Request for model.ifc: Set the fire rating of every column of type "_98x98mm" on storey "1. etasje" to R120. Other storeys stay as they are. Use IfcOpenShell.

First a look at what the model holds.

```python
import ifcopenshell
import ifcopenshell.util.element

model = ifcopenshell.open("model.ifc")
print(model.schema)
storey = next(s for s in model.by_type("IfcBuildingStorey") if s.Name == "1. etasje")
columns = [e for e in ifcopenshell.util.element.get_decomposition(storey) if e.is_a("IfcColumn")]
seen = {}
for e in columns:
    element_type = ifcopenshell.util.element.get_type(e)
    key = (element_type.Name if element_type != e and element_type else None, ifcopenshell.util.element.get_pset(e, "Pset_ColumnCommon", "FireRating"))
    seen[key] = seen.get(key, 0) + 1
for (name, value), count in sorted(seen.items(), key=str):
    print(count, "x", name, "|", value)
```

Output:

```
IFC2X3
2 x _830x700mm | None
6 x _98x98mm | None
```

```python
import ifcopenshell
import ifcopenshell.api.pset
import ifcopenshell.util.element

model = ifcopenshell.open("model.ifc")

storey = next(s for s in model.by_type("IfcBuildingStorey") if s.Name == "1. etasje")
columns = [e for e in ifcopenshell.util.element.get_decomposition(storey) if e.is_a("IfcColumn")]

count = 0
for e in columns:
    element_type = ifcopenshell.util.element.get_type(e)
    if element_type in (None, e) or element_type.Name != "_98x98mm":
        continue
    # add_pset returns the element's existing set when there is one.
    pset = ifcopenshell.api.pset.add_pset(model, product=e, name="Pset_ColumnCommon")
    ifcopenshell.api.pset.edit_pset(model, pset=pset, properties={"FireRating": "R120"})
    count += 1

print(count, "columns updated")

model.write("model_updated.ifc")
```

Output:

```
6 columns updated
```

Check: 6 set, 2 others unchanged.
